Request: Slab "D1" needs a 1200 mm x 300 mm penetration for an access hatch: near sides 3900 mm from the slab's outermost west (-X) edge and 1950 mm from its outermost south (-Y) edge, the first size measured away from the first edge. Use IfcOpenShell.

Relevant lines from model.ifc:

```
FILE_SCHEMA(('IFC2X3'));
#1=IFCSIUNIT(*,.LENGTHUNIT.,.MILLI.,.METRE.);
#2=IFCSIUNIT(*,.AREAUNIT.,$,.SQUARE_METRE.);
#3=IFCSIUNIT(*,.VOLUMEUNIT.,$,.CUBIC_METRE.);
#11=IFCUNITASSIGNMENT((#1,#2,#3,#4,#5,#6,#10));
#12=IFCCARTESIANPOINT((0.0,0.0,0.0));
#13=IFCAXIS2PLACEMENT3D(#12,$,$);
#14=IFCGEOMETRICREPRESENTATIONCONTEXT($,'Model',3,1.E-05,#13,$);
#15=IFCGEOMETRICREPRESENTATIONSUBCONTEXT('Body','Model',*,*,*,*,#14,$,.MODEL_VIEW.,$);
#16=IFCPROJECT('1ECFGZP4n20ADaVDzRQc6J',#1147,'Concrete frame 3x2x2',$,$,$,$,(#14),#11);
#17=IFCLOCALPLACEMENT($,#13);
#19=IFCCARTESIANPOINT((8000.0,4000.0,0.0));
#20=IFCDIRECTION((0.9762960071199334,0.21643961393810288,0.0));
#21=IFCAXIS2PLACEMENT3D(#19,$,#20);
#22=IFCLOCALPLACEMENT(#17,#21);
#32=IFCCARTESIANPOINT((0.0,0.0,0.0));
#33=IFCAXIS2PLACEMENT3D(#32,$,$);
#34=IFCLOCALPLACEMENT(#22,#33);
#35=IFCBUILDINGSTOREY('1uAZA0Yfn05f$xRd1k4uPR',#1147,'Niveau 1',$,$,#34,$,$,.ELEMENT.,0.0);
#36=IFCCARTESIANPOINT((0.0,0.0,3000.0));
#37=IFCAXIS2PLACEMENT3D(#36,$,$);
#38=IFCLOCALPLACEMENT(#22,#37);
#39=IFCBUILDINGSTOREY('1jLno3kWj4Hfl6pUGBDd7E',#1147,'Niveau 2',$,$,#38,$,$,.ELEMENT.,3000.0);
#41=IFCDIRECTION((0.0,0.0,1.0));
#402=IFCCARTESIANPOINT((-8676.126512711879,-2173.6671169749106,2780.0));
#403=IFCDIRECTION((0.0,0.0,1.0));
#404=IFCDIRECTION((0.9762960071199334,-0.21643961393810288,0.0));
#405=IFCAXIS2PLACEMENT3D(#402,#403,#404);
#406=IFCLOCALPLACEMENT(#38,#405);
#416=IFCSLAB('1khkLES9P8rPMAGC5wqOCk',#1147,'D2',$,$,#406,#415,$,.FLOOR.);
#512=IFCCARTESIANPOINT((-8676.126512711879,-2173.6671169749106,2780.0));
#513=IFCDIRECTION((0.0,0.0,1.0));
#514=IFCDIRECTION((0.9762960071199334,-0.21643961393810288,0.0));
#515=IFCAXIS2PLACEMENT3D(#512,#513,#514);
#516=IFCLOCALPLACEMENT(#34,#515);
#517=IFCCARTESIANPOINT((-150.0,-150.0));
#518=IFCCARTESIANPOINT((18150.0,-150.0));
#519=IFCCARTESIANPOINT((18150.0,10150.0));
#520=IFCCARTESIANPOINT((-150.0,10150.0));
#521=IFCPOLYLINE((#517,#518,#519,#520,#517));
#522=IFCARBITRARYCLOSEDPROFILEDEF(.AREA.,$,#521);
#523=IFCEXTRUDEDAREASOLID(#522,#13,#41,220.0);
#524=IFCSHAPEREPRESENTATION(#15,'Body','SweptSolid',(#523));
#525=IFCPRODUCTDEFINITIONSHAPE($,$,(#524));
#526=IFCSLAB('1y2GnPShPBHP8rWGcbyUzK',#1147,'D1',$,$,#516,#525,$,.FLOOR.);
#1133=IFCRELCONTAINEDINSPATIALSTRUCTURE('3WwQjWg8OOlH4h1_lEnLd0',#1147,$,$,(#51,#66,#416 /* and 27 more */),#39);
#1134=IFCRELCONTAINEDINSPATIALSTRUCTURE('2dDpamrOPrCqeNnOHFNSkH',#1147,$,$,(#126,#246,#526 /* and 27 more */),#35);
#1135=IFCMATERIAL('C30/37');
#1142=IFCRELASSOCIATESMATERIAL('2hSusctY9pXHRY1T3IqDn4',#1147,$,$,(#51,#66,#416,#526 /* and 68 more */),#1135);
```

```python
import numpy as np
import ifcopenshell
import ifcopenshell.api.feature
import ifcopenshell.api.geometry
import ifcopenshell.api.root
import ifcopenshell.geom
import ifcopenshell.util.placement
import ifcopenshell.util.representation
import ifcopenshell.util.shape
import ifcopenshell.util.unit

model = ifcopenshell.open("model.ifc")
unit_scale = ifcopenshell.util.unit.calculate_unit_scale(model)
settings = ifcopenshell.geom.settings()


def volume(element):
    """Net volume in cubic metres, openings subtracted."""
    shape = ifcopenshell.geom.create_shape(settings, element)
    return ifcopenshell.util.shape.get_volume(shape.geometry)


slab = model.by_guid("1y2GnPShPBHP8rWGcbyUzK")
before = volume(slab)

# Extent in the slab's own axes, in metres. The edges named are its -X and -Y sides.
slab_shape = ifcopenshell.geom.create_shape(settings, slab)
vertices = ifcopenshell.util.shape.get_vertices(slab_shape.geometry)
x_min, y_min, bottom = vertices.min(axis=0)
top = vertices[:, 2].max()

opening = ifcopenshell.api.root.create_entity(model, ifc_class="IfcOpeningElement", name="Access hatch opening")
context = ifcopenshell.util.representation.get_context(model, "Model", "Body", "MODEL_VIEW")
width, depth = 1.2, 0.3
outline = [(0.0, 0.0), (width, 0.0), (width, depth), (0.0, depth), (0.0, 0.0)]
# Overshoot both faces by 50 mm so the cut is clean.
shape = ifcopenshell.api.geometry.add_slab_representation(
    model, context=context, depth=top - bottom + 0.1, polyline=outline
)
ifcopenshell.api.geometry.assign_representation(model, product=opening, representation=shape)

matrix = ifcopenshell.util.placement.get_local_placement(slab.ObjectPlacement)
matrix[:, 3] = matrix @ np.append(np.array([x_min + 3.9, y_min + 1.95, bottom - 0.05]) / unit_scale, 1.0)
ifcopenshell.api.geometry.edit_object_placement(model, product=opening, matrix=matrix, is_si=False)
ifcopenshell.api.feature.add_feature(model, feature=opening, element=slab)

after = volume(slab)

print(f"slab volume {before:.3f} -> {after:.3f} m3")

model.write("model_rev.ifc")
```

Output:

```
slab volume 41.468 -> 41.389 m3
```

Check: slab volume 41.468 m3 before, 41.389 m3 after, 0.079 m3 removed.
